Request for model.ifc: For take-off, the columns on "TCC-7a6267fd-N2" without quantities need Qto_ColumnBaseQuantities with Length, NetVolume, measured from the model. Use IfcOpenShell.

First a look at what the model holds.

```python
import ifcopenshell
import ifcopenshell.util.element
import ifcopenshell.util.unit

model = ifcopenshell.open("model.ifc")
print(model.schema)
for unit_type in ("LENGTHUNIT", "AREAUNIT", "VOLUMEUNIT"):
    print(unit_type, ifcopenshell.util.unit.calculate_unit_scale(model, unit_type))
storey = next(s for s in model.by_type("IfcBuildingStorey") if s.Name == "TCC-7a6267fd-N2")
columns = [e for e in ifcopenshell.util.element.get_decomposition(storey) if e.is_a("IfcColumn")]
for e in sorted(columns, key=lambda e: e.id()):
    print(e.id(), e.is_a(), e.Name, list(ifcopenshell.util.element.get_psets(e, qtos_only=True)), sep=" | ")
```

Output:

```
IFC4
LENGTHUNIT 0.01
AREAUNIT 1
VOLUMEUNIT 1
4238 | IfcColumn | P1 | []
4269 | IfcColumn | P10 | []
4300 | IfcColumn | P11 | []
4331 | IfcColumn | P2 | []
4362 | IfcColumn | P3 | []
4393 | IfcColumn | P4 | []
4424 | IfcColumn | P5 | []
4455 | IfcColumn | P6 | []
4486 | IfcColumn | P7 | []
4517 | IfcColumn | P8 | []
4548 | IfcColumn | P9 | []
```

```python
import ifcopenshell
import ifcopenshell.api.pset
import ifcopenshell.geom
import ifcopenshell.util.element
import ifcopenshell.util.shape
import ifcopenshell.util.unit

model = ifcopenshell.open("model.ifc")
unit_scale = ifcopenshell.util.unit.calculate_unit_scale(model)
volume_scale = ifcopenshell.util.unit.calculate_unit_scale(model, "VOLUMEUNIT")
settings = ifcopenshell.geom.settings()

storey = next(s for s in model.by_type("IfcBuildingStorey") if s.Name == "TCC-7a6267fd-N2")
columns = [e for e in ifcopenshell.util.element.get_decomposition(storey) if e.is_a("IfcColumn")]

for e in sorted(columns, key=lambda e: e.id()):
    if ifcopenshell.util.element.get_psets(e, qtos_only=True, should_inherit=False):
        continue
    # Geometry comes back in metres, in the element's own axes.
    shape = ifcopenshell.geom.create_shape(settings, e)
    values = {
        "Length": ifcopenshell.util.shape.get_z(shape.geometry) / unit_scale,
        "NetVolume": ifcopenshell.util.shape.get_volume(shape.geometry) / volume_scale,
    }
    qto = ifcopenshell.api.pset.add_qto(model, product=e, name="Qto_ColumnBaseQuantities")
    ifcopenshell.api.pset.edit_qto(model, qto=qto, properties=values)
    print(e.id(), {k: round(v, 3) for k, v in values.items()})

model.write("model_v2.ifc")
```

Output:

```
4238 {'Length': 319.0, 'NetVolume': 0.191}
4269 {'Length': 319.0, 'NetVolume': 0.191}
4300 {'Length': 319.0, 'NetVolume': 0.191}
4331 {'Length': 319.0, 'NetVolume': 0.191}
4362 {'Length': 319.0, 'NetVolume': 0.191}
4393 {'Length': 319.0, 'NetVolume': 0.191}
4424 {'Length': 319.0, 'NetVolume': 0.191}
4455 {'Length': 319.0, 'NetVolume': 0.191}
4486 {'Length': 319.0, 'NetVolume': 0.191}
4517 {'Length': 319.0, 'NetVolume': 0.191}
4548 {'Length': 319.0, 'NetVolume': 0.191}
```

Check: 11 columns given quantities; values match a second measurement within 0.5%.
